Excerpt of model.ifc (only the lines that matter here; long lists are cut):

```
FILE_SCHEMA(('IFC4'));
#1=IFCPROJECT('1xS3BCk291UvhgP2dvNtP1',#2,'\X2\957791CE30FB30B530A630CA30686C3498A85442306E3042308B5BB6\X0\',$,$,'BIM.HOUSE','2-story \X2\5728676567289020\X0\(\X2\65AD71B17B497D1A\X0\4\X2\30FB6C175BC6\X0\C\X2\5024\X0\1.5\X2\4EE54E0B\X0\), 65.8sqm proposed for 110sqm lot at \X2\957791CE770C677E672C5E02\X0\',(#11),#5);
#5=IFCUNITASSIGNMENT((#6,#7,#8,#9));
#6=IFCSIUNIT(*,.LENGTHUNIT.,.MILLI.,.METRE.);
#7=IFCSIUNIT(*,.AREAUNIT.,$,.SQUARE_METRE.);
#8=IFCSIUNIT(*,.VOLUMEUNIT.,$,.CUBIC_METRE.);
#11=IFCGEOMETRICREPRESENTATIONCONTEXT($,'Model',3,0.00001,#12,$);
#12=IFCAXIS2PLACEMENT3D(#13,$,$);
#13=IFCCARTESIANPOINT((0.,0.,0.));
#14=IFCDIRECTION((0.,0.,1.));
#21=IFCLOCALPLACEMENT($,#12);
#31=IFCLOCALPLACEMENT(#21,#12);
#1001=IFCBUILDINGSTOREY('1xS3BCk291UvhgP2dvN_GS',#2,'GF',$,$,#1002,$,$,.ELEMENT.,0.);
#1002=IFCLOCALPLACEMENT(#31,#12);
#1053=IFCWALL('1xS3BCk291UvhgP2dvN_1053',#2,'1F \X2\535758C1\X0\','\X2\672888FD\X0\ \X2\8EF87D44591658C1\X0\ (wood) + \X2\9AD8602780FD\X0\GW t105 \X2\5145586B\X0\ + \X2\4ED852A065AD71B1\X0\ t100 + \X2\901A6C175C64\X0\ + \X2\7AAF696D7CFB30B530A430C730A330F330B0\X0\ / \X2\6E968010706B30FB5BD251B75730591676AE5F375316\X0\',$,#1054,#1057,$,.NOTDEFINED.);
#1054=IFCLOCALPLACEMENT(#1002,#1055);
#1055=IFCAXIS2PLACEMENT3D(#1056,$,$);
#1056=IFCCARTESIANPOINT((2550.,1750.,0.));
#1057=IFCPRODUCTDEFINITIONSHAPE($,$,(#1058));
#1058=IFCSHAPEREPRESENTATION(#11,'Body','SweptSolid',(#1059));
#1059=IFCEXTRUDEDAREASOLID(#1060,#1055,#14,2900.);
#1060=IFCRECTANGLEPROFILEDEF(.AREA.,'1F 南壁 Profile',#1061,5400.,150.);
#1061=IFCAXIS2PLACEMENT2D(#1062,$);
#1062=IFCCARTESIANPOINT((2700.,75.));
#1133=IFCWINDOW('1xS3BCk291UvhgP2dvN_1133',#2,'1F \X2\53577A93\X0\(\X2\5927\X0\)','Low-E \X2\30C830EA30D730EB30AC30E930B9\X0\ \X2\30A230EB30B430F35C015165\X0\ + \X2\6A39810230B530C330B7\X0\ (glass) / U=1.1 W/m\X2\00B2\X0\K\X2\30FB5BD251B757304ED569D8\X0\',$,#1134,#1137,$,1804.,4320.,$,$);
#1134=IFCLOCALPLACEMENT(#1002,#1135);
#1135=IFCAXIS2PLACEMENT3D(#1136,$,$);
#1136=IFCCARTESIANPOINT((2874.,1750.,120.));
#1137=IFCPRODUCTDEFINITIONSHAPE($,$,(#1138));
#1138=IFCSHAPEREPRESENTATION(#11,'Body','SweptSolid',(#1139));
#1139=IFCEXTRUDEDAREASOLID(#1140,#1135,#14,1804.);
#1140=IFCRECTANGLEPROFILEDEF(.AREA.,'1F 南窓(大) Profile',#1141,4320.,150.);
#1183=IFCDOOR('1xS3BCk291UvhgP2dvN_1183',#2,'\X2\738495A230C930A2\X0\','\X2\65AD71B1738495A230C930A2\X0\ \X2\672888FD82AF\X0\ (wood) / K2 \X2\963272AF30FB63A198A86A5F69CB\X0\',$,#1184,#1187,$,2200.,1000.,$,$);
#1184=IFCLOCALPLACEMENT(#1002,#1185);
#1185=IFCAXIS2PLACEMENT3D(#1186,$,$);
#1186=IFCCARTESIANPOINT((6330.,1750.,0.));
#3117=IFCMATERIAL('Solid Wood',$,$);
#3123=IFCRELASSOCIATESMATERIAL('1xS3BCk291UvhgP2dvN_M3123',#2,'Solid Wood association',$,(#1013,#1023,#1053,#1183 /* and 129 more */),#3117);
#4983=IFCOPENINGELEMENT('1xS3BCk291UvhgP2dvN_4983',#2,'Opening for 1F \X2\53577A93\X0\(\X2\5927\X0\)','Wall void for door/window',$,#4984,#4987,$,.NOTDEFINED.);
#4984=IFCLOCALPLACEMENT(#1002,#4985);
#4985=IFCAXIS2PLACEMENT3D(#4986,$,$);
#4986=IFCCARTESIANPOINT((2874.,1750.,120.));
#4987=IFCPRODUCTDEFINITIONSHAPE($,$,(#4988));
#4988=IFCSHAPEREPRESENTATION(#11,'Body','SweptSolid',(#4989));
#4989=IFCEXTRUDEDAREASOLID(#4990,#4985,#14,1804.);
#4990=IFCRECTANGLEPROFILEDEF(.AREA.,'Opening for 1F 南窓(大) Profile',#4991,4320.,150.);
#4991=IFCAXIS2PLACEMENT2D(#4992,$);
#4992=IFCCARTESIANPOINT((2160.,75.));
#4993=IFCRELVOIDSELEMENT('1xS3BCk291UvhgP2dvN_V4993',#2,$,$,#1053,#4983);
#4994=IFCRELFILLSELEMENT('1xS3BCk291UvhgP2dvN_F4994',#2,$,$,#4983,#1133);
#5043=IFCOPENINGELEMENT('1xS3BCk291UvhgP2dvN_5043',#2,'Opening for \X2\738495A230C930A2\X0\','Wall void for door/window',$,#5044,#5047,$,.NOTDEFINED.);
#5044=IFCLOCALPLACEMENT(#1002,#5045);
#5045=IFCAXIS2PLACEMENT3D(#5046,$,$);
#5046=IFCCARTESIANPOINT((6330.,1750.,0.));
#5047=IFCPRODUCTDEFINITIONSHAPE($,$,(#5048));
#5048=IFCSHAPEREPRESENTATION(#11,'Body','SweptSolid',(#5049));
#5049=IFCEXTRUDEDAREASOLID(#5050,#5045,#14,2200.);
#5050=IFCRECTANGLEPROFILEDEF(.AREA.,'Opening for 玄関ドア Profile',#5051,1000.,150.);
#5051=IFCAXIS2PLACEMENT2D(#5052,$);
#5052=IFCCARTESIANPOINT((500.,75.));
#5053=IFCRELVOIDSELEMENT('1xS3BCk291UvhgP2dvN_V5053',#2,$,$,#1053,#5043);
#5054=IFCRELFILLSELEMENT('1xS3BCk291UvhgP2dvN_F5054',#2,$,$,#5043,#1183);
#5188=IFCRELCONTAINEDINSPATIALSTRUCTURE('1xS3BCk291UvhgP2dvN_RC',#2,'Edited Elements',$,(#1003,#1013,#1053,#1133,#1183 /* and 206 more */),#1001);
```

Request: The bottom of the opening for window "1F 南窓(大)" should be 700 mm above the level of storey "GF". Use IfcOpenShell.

```python
import numpy as np
import ifcopenshell
import ifcopenshell.api.geometry
import ifcopenshell.geom
import ifcopenshell.util.element
import ifcopenshell.util.placement
import ifcopenshell.util.shape
import ifcopenshell.util.unit

model = ifcopenshell.open("model.ifc")
unit_scale = ifcopenshell.util.unit.calculate_unit_scale(model)

window = model.by_guid("1xS3BCk291UvhgP2dvN_1133")
opening = window.FillsVoids[0].RelatingOpeningElement
storey = ifcopenshell.util.element.get_container(window, ifc_class="IfcBuildingStorey")
level = ifcopenshell.util.placement.get_local_placement(storey.ObjectPlacement)[2, 3]

# The opening's origin need not be at the sill, so measure its lowest point.
shape = ifcopenshell.geom.create_shape(ifcopenshell.geom.settings(), opening)
bottom = ifcopenshell.util.shape.get_shape_bottom_elevation(shape, shape.geometry) / unit_scale
dz = level + 0.7 / unit_scale - bottom

shift = np.array([0.0, 0.0, dz])
# The window is not placed relative to its opening, so move both.
for product in (opening, window):
    matrix = ifcopenshell.util.placement.get_local_placement(product.ObjectPlacement)
    matrix[:3, 3] += shift
    ifcopenshell.api.geometry.edit_object_placement(model, product=product, matrix=matrix, is_si=False)

print(f"moved by {dz * unit_scale:+.3f} m")

model.write("model_updated.ifc")
```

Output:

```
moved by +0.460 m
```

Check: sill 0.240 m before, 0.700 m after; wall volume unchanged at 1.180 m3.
